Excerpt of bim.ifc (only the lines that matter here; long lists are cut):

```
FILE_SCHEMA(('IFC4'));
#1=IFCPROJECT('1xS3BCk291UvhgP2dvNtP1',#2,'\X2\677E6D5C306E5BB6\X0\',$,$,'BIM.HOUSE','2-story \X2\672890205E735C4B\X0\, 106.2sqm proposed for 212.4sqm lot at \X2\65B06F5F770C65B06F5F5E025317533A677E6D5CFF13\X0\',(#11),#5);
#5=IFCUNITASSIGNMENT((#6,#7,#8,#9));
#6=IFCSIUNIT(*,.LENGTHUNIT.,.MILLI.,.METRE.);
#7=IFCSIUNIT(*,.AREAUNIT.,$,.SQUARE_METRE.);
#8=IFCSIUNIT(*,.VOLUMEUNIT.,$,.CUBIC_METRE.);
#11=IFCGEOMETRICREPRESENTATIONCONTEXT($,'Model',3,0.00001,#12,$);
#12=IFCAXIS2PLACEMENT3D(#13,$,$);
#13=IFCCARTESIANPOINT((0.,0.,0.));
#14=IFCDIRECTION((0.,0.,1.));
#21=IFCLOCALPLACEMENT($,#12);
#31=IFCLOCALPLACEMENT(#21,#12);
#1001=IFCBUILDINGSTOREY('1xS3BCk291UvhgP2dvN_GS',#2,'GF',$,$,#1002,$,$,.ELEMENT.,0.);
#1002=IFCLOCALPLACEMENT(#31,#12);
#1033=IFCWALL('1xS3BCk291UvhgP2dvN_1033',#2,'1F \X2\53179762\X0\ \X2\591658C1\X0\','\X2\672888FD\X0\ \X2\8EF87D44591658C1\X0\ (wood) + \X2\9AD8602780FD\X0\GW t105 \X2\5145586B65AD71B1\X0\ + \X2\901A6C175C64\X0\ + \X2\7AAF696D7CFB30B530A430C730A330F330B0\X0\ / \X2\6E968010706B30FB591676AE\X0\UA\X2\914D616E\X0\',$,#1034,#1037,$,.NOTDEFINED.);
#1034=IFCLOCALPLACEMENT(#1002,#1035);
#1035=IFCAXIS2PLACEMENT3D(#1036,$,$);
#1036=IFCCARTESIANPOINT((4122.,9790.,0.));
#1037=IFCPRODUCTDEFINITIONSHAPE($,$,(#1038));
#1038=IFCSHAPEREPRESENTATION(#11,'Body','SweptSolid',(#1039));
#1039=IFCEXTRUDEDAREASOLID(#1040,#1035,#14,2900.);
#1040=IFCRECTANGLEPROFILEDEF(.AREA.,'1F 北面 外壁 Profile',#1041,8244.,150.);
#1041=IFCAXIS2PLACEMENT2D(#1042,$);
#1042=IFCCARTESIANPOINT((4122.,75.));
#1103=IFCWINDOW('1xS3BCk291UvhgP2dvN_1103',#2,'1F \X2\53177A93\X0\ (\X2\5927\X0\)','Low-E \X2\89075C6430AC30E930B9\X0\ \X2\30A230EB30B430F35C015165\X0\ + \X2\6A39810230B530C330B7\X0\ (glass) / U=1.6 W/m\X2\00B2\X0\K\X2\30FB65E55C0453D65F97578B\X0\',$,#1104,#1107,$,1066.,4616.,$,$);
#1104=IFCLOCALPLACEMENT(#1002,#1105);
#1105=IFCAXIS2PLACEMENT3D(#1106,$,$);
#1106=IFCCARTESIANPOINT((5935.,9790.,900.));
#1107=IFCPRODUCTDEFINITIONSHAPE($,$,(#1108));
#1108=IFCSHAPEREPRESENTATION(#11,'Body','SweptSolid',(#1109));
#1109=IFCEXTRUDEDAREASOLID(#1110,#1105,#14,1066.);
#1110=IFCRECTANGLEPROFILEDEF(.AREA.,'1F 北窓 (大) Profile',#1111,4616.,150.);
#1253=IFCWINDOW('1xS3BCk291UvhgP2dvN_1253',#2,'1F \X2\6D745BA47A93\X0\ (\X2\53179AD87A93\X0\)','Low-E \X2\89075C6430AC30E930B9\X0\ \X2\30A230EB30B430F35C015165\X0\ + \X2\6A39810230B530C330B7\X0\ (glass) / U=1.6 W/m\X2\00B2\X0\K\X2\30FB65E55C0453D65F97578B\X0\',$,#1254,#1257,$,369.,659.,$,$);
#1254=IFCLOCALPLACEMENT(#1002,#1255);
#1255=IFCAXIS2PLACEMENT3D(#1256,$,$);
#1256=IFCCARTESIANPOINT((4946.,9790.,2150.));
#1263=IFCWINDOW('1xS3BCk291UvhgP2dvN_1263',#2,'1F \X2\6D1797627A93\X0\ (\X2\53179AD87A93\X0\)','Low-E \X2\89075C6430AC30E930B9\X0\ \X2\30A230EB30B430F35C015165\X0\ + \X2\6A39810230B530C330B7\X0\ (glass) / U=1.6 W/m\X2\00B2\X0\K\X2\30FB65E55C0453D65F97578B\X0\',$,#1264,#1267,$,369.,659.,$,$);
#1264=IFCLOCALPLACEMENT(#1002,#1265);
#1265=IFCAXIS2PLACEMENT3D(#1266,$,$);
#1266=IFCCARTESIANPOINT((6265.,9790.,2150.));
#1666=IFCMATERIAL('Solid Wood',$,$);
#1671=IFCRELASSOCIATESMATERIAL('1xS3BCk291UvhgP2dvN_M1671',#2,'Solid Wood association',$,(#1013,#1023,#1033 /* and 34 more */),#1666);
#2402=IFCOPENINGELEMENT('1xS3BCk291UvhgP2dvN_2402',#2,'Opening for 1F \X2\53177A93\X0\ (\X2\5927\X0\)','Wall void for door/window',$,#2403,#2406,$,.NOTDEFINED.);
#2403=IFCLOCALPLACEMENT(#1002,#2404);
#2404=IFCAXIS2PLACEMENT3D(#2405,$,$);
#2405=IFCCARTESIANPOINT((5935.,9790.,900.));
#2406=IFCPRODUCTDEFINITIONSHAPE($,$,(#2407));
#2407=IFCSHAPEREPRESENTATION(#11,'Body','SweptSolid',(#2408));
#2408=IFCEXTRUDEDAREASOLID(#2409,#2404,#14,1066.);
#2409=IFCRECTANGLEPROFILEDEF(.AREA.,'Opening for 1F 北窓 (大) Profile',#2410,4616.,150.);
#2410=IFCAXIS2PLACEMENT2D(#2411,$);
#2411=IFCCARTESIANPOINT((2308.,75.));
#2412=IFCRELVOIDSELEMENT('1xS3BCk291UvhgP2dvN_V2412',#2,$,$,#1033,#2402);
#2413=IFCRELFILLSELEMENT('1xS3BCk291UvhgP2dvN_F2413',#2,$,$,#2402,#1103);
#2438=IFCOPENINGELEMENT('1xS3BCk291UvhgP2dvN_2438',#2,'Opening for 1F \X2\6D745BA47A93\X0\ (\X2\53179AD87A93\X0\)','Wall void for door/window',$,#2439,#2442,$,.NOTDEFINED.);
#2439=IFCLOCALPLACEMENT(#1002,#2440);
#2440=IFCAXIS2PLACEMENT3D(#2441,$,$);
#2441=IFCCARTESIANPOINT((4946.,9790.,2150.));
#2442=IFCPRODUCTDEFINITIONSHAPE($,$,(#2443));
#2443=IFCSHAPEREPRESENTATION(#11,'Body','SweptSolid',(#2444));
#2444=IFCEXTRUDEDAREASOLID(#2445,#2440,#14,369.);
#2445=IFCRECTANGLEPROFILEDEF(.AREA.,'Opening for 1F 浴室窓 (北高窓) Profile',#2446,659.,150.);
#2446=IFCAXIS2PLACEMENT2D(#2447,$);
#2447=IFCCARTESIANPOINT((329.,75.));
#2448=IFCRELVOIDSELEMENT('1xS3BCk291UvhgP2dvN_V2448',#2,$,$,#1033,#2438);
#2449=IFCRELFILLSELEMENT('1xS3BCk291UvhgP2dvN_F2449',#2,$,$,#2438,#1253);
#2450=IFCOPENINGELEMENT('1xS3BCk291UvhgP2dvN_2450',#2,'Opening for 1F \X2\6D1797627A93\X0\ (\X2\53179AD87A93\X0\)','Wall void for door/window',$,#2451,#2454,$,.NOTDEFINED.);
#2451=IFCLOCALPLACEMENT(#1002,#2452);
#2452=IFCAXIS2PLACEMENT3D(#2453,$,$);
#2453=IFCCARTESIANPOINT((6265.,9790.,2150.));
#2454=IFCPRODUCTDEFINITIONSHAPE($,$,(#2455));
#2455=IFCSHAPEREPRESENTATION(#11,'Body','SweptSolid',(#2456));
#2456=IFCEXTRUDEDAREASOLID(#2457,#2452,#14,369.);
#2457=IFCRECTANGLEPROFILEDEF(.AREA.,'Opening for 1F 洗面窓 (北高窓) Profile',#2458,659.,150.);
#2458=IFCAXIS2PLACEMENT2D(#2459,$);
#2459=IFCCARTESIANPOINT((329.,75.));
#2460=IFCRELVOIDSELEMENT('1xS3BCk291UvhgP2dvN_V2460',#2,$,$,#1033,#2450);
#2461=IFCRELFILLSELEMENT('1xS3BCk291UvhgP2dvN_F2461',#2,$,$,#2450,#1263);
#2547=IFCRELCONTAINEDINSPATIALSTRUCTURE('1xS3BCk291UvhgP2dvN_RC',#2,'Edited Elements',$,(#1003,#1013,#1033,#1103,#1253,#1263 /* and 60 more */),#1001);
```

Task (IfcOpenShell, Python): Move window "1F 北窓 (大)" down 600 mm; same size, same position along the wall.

```python
import numpy as np
import ifcopenshell
import ifcopenshell.api.geometry
import ifcopenshell.util.placement
import ifcopenshell.util.unit

model = ifcopenshell.open("bim.ifc")
unit_scale = ifcopenshell.util.unit.calculate_unit_scale(model)

window = model.by_guid("1xS3BCk291UvhgP2dvN_1103")
opening = window.FillsVoids[0].RelatingOpeningElement
dz = -0.6 / unit_scale

shift = np.array([0.0, 0.0, dz])
# The window is not placed relative to its opening, so move both.
for product in (opening, window):
    matrix = ifcopenshell.util.placement.get_local_placement(product.ObjectPlacement)
    matrix[:3, 3] += shift
    ifcopenshell.api.geometry.edit_object_placement(model, product=product, matrix=matrix, is_si=False)

print(f"moved by {dz * unit_scale:+.3f} m")

model.write("bim_v2.ifc")
```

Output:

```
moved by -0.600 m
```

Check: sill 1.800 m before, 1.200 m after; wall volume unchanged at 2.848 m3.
